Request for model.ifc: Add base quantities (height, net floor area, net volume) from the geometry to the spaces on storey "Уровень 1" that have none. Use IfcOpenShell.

First a look at what the model holds.

```python
import ifcopenshell
import ifcopenshell.util.element
import ifcopenshell.util.unit

model = ifcopenshell.open("model.ifc")
print(model.schema)
for unit_type in ("LENGTHUNIT", "AREAUNIT", "VOLUMEUNIT"):
    print(unit_type, ifcopenshell.util.unit.calculate_unit_scale(model, unit_type))
storey = next(s for s in model.by_type("IfcBuildingStorey") if s.Name == "Уровень 1")
spaces = [e for e in ifcopenshell.util.element.get_decomposition(storey) if e.is_a("IfcSpace")]
for e in sorted(spaces, key=lambda e: e.id()):
    print(e.id(), e.is_a(), e.Name, list(ifcopenshell.util.element.get_psets(e, qtos_only=True)), sep=" | ")
```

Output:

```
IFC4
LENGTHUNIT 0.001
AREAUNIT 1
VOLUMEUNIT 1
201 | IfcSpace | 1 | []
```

```python
import ifcopenshell
import ifcopenshell.api.pset
import ifcopenshell.geom
import ifcopenshell.util.element
import ifcopenshell.util.shape
import ifcopenshell.util.unit

model = ifcopenshell.open("model.ifc")
unit_scale = ifcopenshell.util.unit.calculate_unit_scale(model)
area_scale = ifcopenshell.util.unit.calculate_unit_scale(model, "AREAUNIT")
volume_scale = ifcopenshell.util.unit.calculate_unit_scale(model, "VOLUMEUNIT")
settings = ifcopenshell.geom.settings()

storey = next(s for s in model.by_type("IfcBuildingStorey") if s.Name == "Уровень 1")
spaces = [e for e in ifcopenshell.util.element.get_decomposition(storey) if e.is_a("IfcSpace")]

for e in sorted(spaces, key=lambda e: e.id()):
    if ifcopenshell.util.element.get_psets(e, qtos_only=True, should_inherit=False):
        continue
    # Geometry comes back in metres, in the element's own axes.
    shape = ifcopenshell.geom.create_shape(settings, e)
    values = {
        "Height": ifcopenshell.util.shape.get_z(shape.geometry) / unit_scale,
        "NetFloorArea": ifcopenshell.util.shape.get_footprint_area(shape.geometry) / area_scale,
        "NetVolume": ifcopenshell.util.shape.get_volume(shape.geometry) / volume_scale,
    }
    qto = ifcopenshell.api.pset.add_qto(model, product=e, name="Qto_SpaceBaseQuantities")
    ifcopenshell.api.pset.edit_qto(model, qto=qto, properties=values)
    print(e.id(), {k: round(v, 3) for k, v in values.items()})

model.write("model_v2.ifc")
```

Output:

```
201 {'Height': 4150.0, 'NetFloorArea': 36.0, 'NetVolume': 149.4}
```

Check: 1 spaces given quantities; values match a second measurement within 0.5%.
